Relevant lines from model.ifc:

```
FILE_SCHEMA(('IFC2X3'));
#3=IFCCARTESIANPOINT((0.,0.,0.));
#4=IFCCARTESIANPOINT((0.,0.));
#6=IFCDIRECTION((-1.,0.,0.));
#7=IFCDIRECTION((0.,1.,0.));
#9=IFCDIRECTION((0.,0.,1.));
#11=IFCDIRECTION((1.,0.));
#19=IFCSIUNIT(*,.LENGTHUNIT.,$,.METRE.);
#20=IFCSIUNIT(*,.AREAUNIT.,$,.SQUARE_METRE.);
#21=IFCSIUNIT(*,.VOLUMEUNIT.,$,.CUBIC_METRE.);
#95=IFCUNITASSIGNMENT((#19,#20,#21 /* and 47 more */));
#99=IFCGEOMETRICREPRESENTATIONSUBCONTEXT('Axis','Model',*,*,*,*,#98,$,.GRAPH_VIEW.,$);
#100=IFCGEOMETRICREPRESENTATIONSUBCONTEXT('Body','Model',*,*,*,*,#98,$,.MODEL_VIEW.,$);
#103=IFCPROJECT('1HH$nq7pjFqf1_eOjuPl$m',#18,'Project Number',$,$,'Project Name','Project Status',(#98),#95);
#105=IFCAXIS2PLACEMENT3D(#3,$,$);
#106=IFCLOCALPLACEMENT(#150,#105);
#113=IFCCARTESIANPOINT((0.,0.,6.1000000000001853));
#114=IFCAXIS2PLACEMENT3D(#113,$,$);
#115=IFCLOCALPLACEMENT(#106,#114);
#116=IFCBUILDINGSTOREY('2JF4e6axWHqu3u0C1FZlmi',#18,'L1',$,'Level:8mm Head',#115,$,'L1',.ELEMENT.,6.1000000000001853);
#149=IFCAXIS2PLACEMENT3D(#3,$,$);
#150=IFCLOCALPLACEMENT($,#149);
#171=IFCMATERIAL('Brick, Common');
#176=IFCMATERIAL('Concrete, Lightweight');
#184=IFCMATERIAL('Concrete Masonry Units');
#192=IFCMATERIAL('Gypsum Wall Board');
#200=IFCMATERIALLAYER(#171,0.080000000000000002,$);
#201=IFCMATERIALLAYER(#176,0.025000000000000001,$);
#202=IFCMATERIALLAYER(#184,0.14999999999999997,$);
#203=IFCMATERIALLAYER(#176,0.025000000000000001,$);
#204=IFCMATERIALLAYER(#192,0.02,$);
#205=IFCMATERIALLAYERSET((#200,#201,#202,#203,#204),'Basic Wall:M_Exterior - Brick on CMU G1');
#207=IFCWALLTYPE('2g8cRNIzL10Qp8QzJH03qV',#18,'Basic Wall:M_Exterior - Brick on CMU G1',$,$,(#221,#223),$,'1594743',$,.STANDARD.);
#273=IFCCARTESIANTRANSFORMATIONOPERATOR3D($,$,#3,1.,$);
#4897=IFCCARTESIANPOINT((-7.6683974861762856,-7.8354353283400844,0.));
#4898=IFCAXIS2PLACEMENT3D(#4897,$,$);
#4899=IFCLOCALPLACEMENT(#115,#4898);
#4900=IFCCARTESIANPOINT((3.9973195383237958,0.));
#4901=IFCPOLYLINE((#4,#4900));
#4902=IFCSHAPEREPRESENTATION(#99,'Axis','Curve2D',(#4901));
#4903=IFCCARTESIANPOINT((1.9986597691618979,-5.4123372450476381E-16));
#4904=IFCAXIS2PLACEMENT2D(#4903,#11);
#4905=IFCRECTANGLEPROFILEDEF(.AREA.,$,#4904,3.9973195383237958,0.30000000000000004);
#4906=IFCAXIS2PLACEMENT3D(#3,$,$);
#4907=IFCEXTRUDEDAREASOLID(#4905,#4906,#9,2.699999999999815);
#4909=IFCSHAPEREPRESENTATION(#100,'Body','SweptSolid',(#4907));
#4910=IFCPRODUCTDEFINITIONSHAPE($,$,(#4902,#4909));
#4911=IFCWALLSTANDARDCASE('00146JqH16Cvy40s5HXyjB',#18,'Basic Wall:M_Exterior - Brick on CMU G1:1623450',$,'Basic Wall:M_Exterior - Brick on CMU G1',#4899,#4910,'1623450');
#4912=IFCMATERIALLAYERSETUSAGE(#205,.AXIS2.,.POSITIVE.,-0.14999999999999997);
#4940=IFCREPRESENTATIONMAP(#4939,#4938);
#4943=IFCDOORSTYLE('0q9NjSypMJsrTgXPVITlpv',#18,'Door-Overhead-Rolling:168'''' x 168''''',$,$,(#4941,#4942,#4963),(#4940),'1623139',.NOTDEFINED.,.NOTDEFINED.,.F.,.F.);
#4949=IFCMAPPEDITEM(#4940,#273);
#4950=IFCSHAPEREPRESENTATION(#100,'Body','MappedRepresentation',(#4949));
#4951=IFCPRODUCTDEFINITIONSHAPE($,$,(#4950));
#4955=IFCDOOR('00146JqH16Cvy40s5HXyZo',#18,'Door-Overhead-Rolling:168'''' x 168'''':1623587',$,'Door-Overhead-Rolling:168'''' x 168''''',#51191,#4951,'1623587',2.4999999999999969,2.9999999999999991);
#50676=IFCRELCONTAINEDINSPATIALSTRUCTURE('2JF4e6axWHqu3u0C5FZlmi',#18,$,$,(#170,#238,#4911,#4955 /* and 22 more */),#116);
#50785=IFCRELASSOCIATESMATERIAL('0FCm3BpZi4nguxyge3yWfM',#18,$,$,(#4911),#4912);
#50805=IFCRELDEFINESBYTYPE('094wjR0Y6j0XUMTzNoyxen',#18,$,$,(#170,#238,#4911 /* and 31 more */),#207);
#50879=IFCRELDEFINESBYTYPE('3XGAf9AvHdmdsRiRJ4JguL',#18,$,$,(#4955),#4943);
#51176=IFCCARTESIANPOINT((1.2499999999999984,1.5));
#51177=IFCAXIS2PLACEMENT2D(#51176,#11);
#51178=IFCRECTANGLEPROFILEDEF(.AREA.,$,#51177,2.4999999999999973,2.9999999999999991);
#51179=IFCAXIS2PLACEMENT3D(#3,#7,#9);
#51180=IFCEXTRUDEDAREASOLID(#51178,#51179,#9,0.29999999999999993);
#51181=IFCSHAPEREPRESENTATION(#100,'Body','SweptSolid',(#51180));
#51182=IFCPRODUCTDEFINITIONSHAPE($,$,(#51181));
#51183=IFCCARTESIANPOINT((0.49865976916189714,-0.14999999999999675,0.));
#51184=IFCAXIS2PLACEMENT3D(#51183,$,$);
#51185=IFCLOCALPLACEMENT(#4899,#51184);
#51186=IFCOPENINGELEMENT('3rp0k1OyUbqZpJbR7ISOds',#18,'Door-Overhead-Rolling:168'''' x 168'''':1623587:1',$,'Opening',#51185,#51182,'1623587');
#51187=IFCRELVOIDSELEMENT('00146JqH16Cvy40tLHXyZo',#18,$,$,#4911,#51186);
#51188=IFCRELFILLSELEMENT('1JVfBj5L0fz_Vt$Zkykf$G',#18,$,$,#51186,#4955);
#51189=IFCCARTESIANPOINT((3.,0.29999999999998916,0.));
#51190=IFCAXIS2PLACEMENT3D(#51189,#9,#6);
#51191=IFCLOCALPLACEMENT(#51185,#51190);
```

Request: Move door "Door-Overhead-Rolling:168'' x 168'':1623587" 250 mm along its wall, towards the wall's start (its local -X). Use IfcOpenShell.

```python
import ifcopenshell
import ifcopenshell.api.geometry
import ifcopenshell.util.placement

model = ifcopenshell.open("model.ifc")

door = model.by_id(4955)
opening = door.FillsVoids[0].RelatingOpeningElement
wall = opening.VoidsElements[0].RelatingBuildingElement

wall_matrix = ifcopenshell.util.placement.get_local_placement(wall.ObjectPlacement)
shift = wall_matrix[:3, 0] * -0.25
before = ifcopenshell.util.placement.get_local_placement(door.ObjectPlacement)[:3, 3].copy()

# The door is placed relative to its opening, so it follows when the opening moves.
matrix = ifcopenshell.util.placement.get_local_placement(opening.ObjectPlacement)
matrix[:3, 3] += shift
ifcopenshell.api.geometry.edit_object_placement(
    model, product=opening, matrix=matrix, is_si=False, should_transform_children=True
)

after = ifcopenshell.util.placement.get_local_placement(door.ObjectPlacement)[:3, 3]
print("door moved by", (after - before).round(3) + 0.0)

model.write("model_edited.ifc")
```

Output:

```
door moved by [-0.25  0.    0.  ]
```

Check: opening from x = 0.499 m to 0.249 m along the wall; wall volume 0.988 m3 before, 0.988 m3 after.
